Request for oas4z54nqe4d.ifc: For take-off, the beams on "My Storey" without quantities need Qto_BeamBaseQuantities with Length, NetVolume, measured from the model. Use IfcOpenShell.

First a look at what the model holds.

```python
import ifcopenshell
import ifcopenshell.util.element
import ifcopenshell.util.unit

model = ifcopenshell.open("oas4z54nqe4d.ifc")
print(model.schema)
for unit_type in ("LENGTHUNIT", "AREAUNIT", "VOLUMEUNIT"):
    print(unit_type, ifcopenshell.util.unit.calculate_unit_scale(model, unit_type))
storey = next(s for s in model.by_type("IfcBuildingStorey") if s.Name == "My Storey")
beams = [e for e in ifcopenshell.util.element.get_decomposition(storey) if e.is_a("IfcBeam")]
for e in sorted(beams, key=lambda e: e.id()):
    print(e.id(), e.is_a(), e.Name, list(ifcopenshell.util.element.get_psets(e, qtos_only=True)), sep=" | ")
```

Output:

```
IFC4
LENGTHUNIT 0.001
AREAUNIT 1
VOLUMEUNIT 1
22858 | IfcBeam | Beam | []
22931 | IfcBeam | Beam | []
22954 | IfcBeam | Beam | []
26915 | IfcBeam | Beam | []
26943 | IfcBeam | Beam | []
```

```python
import ifcopenshell
import ifcopenshell.api.pset
import ifcopenshell.geom
import ifcopenshell.util.element
import ifcopenshell.util.shape
import ifcopenshell.util.unit

model = ifcopenshell.open("oas4z54nqe4d.ifc")
unit_scale = ifcopenshell.util.unit.calculate_unit_scale(model)
volume_scale = ifcopenshell.util.unit.calculate_unit_scale(model, "VOLUMEUNIT")
settings = ifcopenshell.geom.settings()

storey = next(s for s in model.by_type("IfcBuildingStorey") if s.Name == "My Storey")
beams = [e for e in ifcopenshell.util.element.get_decomposition(storey) if e.is_a("IfcBeam")]

for e in sorted(beams, key=lambda e: e.id()):
    if ifcopenshell.util.element.get_psets(e, qtos_only=True, should_inherit=False):
        continue
    # Geometry comes back in metres, in the element's own axes.
    shape = ifcopenshell.geom.create_shape(settings, e)
    values = {
        "Length": ifcopenshell.util.shape.get_max_xyz(shape.geometry) / unit_scale,
        "NetVolume": ifcopenshell.util.shape.get_volume(shape.geometry) / volume_scale,
    }
    qto = ifcopenshell.api.pset.add_qto(model, product=e, name="Qto_BeamBaseQuantities")
    ifcopenshell.api.pset.edit_qto(model, qto=qto, properties=values)
    print(e.id(), {k: round(v, 3) for k, v in values.items()})

model.write("oas4z54nqe4d-out.ifc")
```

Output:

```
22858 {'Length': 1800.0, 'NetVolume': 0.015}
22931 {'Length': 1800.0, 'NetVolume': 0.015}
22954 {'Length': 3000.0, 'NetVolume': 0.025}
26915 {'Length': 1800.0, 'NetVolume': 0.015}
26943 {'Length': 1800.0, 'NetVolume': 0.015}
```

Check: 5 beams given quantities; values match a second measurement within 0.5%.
